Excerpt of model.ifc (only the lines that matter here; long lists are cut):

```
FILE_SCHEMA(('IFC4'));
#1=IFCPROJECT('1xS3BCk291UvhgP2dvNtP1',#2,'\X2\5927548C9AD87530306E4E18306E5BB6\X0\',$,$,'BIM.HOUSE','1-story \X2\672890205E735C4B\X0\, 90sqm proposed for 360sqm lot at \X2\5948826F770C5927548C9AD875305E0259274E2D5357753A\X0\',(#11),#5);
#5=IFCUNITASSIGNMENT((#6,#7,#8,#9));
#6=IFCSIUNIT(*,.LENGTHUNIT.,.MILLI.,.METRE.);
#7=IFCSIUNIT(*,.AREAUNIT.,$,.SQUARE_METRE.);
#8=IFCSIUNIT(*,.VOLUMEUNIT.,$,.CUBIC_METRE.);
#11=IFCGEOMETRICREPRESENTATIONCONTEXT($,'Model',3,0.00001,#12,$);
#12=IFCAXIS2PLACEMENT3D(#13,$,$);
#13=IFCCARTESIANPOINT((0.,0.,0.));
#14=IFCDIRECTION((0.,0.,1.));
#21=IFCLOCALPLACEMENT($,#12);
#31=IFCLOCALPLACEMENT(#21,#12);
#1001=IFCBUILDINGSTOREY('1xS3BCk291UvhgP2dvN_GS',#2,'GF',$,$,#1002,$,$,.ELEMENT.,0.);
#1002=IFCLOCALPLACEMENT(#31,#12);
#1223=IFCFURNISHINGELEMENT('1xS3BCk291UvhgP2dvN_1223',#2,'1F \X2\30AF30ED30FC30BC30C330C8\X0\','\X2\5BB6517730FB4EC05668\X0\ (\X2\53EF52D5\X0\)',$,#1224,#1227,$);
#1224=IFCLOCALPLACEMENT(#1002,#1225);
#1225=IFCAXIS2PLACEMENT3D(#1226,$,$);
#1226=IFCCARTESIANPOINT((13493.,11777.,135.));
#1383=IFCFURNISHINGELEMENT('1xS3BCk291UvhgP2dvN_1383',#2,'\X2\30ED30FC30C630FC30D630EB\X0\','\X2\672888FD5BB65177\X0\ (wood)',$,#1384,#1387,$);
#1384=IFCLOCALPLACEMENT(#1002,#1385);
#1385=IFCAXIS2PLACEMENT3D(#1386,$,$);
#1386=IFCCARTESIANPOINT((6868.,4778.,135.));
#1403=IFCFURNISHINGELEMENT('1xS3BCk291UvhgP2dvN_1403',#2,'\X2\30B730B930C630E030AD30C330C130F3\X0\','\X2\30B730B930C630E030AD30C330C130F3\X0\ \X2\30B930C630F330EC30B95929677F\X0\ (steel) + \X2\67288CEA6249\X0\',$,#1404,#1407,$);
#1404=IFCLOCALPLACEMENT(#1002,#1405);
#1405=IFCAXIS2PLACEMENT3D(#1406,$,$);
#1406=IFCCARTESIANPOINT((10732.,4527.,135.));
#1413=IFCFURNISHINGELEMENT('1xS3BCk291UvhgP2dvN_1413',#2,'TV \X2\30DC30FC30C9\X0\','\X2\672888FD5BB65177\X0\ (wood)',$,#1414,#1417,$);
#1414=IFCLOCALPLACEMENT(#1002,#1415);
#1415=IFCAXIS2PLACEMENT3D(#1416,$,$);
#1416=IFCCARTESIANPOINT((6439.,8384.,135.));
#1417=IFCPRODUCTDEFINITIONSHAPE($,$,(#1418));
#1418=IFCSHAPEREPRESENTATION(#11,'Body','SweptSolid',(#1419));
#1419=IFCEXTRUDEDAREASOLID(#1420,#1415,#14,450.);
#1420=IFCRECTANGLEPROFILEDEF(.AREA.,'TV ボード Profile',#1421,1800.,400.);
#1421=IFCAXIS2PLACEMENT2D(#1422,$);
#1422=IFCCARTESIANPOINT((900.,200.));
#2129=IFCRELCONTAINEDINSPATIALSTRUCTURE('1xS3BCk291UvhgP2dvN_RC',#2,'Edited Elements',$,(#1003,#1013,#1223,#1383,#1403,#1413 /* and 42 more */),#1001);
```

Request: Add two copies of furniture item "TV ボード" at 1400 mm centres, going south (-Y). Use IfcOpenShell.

```python
import numpy as np
import ifcopenshell
import ifcopenshell.api.geometry
import ifcopenshell.api.root
import ifcopenshell.util.element
import ifcopenshell.util.placement

model = ifcopenshell.open("model.ifc")


def reuse_history(source, copy):
    """copy_class also copies each property set's owner history, people and application; keep the originals."""
    for rel in copy.IsDefinedBy:
        if rel.is_a("IfcRelDefinesByProperties") and (history := rel.RelatingPropertyDefinition.OwnerHistory):
            rel.RelatingPropertyDefinition.OwnerHistory = source.OwnerHistory
            ifcopenshell.util.element.remove_deep2(model, history)


source = model.by_id(1413)
base = ifcopenshell.util.placement.get_local_placement(source.ObjectPlacement)
step = np.array([0.0, -1.0, 0.0]) * 1400.0

for i in range(1, 3):
    copy = ifcopenshell.api.root.copy_class(model, product=source)
    copy.Representation = ifcopenshell.util.element.copy_deep(
        model, source.Representation, exclude=["IfcGeometricRepresentationContext", "IfcRepresentationMap"]
    )
    reuse_history(source, copy)
    matrix = base.copy()
    matrix[:3, 3] += i * step
    print("added at", matrix[:3, 3].round(3) + 0.0)
    ifcopenshell.api.geometry.edit_object_placement(model, product=copy, matrix=matrix, is_si=False)

model.write("model_updated.ifc")
```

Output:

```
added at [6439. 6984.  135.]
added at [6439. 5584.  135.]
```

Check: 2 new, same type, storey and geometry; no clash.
